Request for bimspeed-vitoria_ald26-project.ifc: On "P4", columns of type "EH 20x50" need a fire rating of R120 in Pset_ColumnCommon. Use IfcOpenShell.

First a look at what the model holds.

```python
import ifcopenshell
import ifcopenshell.util.element

model = ifcopenshell.open("bimspeed-vitoria_ald26-project.ifc")
print(model.schema)
storey = next(s for s in model.by_type("IfcBuildingStorey") if s.Name == "P4")
columns = [e for e in ifcopenshell.util.element.get_decomposition(storey) if e.is_a("IfcColumn")]
seen = {}
for e in columns:
    element_type = ifcopenshell.util.element.get_type(e)
    key = (element_type.Name if element_type != e and element_type else None, ifcopenshell.util.element.get_pset(e, "Pset_ColumnCommon", "FireRating"))
    seen[key] = seen.get(key, 0) + 1
for (name, value), count in sorted(seen.items(), key=str):
    print(count, "x", name, "|", value)
```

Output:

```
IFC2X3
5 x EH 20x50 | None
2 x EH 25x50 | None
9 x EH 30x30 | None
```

```python
import ifcopenshell
import ifcopenshell.api.pset
import ifcopenshell.util.element

model = ifcopenshell.open("bimspeed-vitoria_ald26-project.ifc")

storey = next(s for s in model.by_type("IfcBuildingStorey") if s.Name == "P4")
columns = [e for e in ifcopenshell.util.element.get_decomposition(storey) if e.is_a("IfcColumn")]

count = 0
for e in columns:
    element_type = ifcopenshell.util.element.get_type(e)
    if element_type in (None, e) or element_type.Name != "EH 20x50":
        continue
    # add_pset returns the element's existing set when there is one.
    pset = ifcopenshell.api.pset.add_pset(model, product=e, name="Pset_ColumnCommon")
    ifcopenshell.api.pset.edit_pset(model, pset=pset, properties={"FireRating": "R120"})
    count += 1

print(count, "columns updated")

model.write("bimspeed-vitoria_ald26-project-out.ifc")
```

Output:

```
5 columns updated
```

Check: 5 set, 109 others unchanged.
